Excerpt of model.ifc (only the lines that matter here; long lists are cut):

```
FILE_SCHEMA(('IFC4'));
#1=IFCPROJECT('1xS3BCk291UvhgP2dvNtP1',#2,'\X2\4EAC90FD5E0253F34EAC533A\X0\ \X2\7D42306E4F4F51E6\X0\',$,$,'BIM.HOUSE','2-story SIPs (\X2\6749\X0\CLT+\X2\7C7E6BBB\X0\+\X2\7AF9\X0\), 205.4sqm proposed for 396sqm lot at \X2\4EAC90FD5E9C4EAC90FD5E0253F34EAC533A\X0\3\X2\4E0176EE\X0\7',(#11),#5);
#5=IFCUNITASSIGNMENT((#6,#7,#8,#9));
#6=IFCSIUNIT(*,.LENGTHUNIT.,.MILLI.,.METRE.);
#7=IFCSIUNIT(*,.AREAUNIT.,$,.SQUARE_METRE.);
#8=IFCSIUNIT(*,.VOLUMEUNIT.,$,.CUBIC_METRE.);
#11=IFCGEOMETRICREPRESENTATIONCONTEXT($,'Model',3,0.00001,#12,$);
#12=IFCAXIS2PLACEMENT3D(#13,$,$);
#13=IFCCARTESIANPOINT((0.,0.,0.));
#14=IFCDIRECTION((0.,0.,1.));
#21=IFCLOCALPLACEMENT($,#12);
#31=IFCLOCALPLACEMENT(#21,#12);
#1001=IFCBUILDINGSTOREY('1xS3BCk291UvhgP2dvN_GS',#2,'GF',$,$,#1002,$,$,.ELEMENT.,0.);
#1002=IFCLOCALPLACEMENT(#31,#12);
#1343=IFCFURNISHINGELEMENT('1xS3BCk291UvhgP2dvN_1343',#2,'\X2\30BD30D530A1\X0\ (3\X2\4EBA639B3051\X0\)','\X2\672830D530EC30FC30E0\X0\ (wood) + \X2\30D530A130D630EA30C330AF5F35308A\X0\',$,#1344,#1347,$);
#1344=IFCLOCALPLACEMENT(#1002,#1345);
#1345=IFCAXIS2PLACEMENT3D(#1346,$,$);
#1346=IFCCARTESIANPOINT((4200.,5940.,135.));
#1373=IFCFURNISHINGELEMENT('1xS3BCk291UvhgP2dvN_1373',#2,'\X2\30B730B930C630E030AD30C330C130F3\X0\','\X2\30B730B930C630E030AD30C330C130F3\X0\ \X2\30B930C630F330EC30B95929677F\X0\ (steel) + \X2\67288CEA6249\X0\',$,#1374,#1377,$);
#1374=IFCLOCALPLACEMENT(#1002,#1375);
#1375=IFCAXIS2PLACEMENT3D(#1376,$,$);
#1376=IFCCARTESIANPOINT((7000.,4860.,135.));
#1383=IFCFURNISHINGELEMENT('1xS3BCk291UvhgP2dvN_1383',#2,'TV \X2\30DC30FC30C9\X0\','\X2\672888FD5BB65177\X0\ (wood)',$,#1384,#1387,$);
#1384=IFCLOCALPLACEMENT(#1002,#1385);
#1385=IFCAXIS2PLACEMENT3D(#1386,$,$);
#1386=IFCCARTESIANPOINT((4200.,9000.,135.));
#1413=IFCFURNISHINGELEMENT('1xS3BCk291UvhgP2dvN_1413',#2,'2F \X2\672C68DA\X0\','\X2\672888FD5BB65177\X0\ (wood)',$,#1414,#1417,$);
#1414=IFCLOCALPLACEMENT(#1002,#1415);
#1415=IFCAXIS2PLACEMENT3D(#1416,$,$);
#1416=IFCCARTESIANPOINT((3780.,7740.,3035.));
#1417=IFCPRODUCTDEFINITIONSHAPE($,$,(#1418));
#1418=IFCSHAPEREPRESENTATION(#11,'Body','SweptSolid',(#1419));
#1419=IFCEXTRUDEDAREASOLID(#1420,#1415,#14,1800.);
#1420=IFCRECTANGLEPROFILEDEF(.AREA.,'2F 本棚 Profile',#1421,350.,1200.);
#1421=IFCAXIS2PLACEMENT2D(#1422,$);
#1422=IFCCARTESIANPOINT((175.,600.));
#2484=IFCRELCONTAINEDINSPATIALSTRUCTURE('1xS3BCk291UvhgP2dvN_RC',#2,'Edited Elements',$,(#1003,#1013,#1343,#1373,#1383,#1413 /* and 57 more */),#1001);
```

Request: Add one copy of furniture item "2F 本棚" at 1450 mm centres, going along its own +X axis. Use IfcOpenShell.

```python
import ifcopenshell
import ifcopenshell.api.geometry
import ifcopenshell.api.root
import ifcopenshell.util.element
import ifcopenshell.util.placement
import ifcopenshell.util.unit

model = ifcopenshell.open("model.ifc")
unit_scale = ifcopenshell.util.unit.calculate_unit_scale(model)


def reuse_history(source, copy):
    """copy_class also copies each property set's owner history, people and application; keep the originals."""
    for rel in copy.IsDefinedBy:
        if rel.is_a("IfcRelDefinesByProperties") and (history := rel.RelatingPropertyDefinition.OwnerHistory):
            rel.RelatingPropertyDefinition.OwnerHistory = source.OwnerHistory
            ifcopenshell.util.element.remove_deep2(model, history)


source = model.by_guid("1xS3BCk291UvhgP2dvN_1413")
base = ifcopenshell.util.placement.get_local_placement(source.ObjectPlacement)
step = base[:3, 0] * 1.45 / unit_scale

for i in range(1, 2):
    copy = ifcopenshell.api.root.copy_class(model, product=source)
    copy.Representation = ifcopenshell.util.element.copy_deep(
        model, source.Representation, exclude=["IfcGeometricRepresentationContext", "IfcRepresentationMap"]
    )
    reuse_history(source, copy)
    matrix = base.copy()
    matrix[:3, 3] += i * step
    print("added at", matrix[:3, 3].round(3) + 0.0)
    ifcopenshell.api.geometry.edit_object_placement(model, product=copy, matrix=matrix, is_si=False)

model.write("model_v2.ifc")
```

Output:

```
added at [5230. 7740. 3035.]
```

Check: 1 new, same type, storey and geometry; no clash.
